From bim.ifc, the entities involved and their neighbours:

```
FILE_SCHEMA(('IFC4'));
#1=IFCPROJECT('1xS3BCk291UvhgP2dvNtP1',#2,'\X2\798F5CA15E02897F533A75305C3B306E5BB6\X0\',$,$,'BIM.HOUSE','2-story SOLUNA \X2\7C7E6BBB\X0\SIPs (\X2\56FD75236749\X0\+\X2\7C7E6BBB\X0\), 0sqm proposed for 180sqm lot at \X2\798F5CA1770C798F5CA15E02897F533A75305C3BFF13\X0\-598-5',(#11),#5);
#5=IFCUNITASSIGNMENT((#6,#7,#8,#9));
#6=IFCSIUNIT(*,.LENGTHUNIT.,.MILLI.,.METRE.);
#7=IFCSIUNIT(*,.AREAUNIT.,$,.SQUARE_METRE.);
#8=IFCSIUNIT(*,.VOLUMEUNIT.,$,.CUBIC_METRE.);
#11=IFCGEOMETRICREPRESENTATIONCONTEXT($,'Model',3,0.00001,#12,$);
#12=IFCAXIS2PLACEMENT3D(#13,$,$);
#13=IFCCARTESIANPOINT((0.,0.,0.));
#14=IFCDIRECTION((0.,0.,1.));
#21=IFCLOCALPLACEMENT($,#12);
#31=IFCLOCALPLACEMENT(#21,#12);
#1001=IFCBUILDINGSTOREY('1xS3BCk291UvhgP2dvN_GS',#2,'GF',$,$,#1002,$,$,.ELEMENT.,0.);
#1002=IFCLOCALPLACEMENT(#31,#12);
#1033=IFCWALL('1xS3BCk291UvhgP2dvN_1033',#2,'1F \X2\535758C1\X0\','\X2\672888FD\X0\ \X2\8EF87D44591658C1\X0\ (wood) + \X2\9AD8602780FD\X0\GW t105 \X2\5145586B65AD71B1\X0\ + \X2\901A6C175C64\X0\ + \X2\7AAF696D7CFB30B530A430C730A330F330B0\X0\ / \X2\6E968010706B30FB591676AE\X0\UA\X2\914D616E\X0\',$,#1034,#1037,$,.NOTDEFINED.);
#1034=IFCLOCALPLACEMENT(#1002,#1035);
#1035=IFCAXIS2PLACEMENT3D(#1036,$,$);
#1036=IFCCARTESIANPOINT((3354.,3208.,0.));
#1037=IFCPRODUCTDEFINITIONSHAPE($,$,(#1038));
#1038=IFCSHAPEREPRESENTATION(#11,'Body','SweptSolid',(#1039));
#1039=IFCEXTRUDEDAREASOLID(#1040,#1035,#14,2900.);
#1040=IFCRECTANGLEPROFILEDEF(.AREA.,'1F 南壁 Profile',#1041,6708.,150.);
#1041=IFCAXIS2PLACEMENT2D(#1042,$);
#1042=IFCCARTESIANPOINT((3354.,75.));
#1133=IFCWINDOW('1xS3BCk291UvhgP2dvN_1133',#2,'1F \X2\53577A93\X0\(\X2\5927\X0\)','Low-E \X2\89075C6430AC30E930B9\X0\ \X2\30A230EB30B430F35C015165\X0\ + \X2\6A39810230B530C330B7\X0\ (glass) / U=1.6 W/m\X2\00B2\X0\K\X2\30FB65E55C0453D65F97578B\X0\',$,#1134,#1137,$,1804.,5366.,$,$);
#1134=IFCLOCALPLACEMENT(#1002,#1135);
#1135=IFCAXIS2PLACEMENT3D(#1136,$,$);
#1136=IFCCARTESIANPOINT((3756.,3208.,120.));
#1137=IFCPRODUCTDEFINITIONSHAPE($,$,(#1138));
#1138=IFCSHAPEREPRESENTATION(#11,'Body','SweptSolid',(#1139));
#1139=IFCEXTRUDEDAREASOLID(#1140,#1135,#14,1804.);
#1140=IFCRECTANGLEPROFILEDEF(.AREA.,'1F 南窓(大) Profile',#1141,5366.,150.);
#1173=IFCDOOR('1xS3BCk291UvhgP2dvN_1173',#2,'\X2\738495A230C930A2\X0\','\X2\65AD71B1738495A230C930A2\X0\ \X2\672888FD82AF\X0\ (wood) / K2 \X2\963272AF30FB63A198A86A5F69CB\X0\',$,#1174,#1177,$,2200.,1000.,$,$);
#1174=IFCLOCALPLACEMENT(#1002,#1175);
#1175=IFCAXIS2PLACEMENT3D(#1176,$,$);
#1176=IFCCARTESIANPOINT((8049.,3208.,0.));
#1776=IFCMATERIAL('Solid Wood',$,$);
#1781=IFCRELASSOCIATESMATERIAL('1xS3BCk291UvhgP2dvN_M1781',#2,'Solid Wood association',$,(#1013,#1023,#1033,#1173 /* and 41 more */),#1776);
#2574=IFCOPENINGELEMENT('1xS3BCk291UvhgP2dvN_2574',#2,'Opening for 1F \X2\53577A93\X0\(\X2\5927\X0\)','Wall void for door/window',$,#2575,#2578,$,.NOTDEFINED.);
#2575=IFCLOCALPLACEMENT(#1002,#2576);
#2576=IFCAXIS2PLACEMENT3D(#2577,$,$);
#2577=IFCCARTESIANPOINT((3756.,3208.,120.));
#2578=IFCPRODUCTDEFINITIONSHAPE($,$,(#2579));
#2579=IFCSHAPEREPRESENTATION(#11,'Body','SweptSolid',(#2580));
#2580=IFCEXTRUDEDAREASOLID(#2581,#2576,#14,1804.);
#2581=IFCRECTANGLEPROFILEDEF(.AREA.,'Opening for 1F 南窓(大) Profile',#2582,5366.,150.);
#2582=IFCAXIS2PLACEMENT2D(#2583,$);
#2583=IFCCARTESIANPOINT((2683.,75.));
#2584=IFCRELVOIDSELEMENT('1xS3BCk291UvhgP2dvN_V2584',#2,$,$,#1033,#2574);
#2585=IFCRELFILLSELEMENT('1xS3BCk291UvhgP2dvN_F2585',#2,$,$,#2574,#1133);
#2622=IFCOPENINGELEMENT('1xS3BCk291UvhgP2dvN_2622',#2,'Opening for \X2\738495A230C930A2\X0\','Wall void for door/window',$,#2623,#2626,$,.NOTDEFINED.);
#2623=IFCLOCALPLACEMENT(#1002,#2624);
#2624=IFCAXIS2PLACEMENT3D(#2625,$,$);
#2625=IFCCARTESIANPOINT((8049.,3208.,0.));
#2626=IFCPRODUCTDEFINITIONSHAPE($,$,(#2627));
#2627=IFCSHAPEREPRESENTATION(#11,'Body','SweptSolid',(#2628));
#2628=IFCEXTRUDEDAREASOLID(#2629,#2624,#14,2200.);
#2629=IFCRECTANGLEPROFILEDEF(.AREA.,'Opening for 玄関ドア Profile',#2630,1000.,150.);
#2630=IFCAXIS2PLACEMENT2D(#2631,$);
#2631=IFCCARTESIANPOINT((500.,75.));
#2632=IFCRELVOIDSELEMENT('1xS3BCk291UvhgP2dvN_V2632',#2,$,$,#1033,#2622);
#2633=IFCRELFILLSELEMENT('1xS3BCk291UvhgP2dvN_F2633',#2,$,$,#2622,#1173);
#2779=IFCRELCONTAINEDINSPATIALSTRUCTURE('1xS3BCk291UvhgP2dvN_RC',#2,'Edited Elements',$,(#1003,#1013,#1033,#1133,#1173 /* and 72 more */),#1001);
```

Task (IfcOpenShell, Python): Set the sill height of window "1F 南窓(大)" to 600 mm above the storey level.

```python
import numpy as np
import ifcopenshell
import ifcopenshell.api.geometry
import ifcopenshell.geom
import ifcopenshell.util.element
import ifcopenshell.util.placement
import ifcopenshell.util.shape
import ifcopenshell.util.unit

model = ifcopenshell.open("bim.ifc")
unit_scale = ifcopenshell.util.unit.calculate_unit_scale(model)

window = model.by_guid("1xS3BCk291UvhgP2dvN_1133")
opening = window.FillsVoids[0].RelatingOpeningElement
storey = ifcopenshell.util.element.get_container(window, ifc_class="IfcBuildingStorey")
level = ifcopenshell.util.placement.get_local_placement(storey.ObjectPlacement)[2, 3]

# The opening's origin need not be at the sill, so measure its lowest point.
shape = ifcopenshell.geom.create_shape(ifcopenshell.geom.settings(), opening)
bottom = ifcopenshell.util.shape.get_shape_bottom_elevation(shape, shape.geometry) / unit_scale
dz = level + 600.0 - bottom

shift = np.array([0.0, 0.0, dz])
# The window is not placed relative to its opening, so move both.
for product in (opening, window):
    matrix = ifcopenshell.util.placement.get_local_placement(product.ObjectPlacement)
    matrix[:3, 3] += shift
    ifcopenshell.api.geometry.edit_object_placement(model, product=product, matrix=matrix, is_si=False)

print(f"moved by {dz * unit_scale:+.3f} m")

model.write("bim_v2.ifc")
```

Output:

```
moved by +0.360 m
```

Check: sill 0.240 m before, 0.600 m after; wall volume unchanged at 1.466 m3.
